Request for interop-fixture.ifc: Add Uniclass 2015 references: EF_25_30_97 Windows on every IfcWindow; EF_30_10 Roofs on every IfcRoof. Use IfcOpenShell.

First a look at what the model holds.

```python
import ifcopenshell

model = ifcopenshell.open("interop-fixture.ifc")
print(model.schema)
print("classifications:", [c.Name for c in model.by_type("IfcClassification")])
for ifc_class in ("IfcDoor", "IfcRoof", "IfcStair", "IfcWall", "IfcWindow"):
    print(ifc_class, len(model.by_type(ifc_class)))
```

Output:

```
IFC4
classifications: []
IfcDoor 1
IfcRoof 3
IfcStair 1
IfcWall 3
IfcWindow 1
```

```python
import ifcopenshell
import ifcopenshell.api.classification

model = ifcopenshell.open("interop-fixture.ifc")

system = ifcopenshell.api.classification.add_classification(model, classification="Uniclass 2015")

codes = {
    "IfcWindow": ("EF_25_30_97", "Windows"),
    "IfcRoof": ("EF_30_10", "Roofs"),
}
for ifc_class, (code, name) in codes.items():
    products = model.by_type(ifc_class)
    ifcopenshell.api.classification.add_reference(
        model, products=products, classification=system, identification=code, name=name
    )
    print(code, len(products))

model.write("interop-fixture_updated.ifc")
```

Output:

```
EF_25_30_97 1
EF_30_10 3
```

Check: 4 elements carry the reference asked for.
